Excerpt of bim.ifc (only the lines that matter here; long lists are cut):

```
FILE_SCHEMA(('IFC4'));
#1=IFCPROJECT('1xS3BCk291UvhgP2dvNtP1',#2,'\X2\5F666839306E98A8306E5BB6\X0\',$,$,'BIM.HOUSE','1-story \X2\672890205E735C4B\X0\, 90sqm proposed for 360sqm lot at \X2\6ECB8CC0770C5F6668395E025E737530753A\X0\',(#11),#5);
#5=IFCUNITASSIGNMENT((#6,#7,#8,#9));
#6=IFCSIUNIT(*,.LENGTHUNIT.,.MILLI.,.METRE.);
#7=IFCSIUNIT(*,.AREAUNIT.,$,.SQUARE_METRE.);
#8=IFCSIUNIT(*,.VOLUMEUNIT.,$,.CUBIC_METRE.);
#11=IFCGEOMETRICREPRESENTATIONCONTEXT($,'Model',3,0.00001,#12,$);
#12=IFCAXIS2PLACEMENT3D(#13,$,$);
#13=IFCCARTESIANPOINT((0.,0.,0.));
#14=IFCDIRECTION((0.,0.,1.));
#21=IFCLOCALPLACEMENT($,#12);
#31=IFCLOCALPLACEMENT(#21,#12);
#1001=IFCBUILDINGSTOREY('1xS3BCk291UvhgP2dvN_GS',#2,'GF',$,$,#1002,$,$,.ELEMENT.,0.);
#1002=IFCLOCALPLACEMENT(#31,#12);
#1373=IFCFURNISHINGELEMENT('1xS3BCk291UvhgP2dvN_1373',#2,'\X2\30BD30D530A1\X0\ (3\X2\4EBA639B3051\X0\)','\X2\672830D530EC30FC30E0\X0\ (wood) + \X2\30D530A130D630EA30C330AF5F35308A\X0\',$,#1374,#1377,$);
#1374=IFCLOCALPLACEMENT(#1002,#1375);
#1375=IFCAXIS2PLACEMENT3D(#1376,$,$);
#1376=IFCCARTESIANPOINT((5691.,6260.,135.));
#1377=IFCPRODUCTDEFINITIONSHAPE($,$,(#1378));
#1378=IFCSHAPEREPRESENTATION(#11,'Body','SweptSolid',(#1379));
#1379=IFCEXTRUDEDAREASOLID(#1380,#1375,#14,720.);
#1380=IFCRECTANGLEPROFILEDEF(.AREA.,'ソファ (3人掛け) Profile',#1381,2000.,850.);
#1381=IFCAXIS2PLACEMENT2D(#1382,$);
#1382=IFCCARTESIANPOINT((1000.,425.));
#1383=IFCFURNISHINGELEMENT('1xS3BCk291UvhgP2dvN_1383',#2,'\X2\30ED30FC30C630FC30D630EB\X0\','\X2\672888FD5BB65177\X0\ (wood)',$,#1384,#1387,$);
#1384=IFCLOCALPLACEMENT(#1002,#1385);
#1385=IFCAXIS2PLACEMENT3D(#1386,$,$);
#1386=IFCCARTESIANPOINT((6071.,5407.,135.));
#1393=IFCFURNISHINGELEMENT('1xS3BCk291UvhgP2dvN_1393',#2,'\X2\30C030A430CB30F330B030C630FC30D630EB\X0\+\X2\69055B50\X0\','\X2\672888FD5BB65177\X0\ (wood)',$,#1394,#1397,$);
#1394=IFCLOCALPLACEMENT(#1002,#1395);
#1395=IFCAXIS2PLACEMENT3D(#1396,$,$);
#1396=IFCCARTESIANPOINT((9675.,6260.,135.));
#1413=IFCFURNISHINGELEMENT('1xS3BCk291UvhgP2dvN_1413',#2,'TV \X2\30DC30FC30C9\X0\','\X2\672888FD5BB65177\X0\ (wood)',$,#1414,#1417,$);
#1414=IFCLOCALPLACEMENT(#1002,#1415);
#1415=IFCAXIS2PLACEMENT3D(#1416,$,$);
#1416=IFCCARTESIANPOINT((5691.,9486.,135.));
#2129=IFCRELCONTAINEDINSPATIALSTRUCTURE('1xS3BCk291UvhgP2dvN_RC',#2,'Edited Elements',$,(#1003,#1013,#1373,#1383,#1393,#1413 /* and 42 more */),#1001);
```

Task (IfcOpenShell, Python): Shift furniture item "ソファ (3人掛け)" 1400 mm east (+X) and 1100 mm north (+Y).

```python
import ifcopenshell
import ifcopenshell.api.geometry
import ifcopenshell.util.placement
import ifcopenshell.util.unit

model = ifcopenshell.open("bim.ifc")
unit_scale = ifcopenshell.util.unit.calculate_unit_scale(model)

item = model.by_guid("1xS3BCk291UvhgP2dvN_1373")
matrix = ifcopenshell.util.placement.get_local_placement(item.ObjectPlacement)
matrix[0, 3] += 1.4 / unit_scale
matrix[1, 3] += 1.1 / unit_scale
ifcopenshell.api.geometry.edit_object_placement(model, product=item, matrix=matrix, is_si=False)

print(ifcopenshell.util.placement.get_local_placement(item.ObjectPlacement).round(3) + 0.0)

model.write("bim-out.ifc")
```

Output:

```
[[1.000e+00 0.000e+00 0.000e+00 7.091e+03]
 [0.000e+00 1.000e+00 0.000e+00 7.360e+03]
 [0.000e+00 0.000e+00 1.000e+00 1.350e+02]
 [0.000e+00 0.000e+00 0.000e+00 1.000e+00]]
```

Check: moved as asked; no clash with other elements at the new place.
